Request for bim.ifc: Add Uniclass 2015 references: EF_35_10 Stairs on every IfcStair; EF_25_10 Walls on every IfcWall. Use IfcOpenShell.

First a look at what the model holds.

```python
import ifcopenshell

model = ifcopenshell.open("bim.ifc")
print(model.schema)
print("classifications:", [c.Name for c in model.by_type("IfcClassification")])
for ifc_class in ("IfcDoor", "IfcRoof", "IfcStair", "IfcWall", "IfcWindow"):
    print(ifc_class, len(model.by_type(ifc_class)))
```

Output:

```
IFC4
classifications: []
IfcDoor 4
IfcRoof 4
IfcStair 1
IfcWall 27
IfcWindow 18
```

```python
import ifcopenshell
import ifcopenshell.api.classification

model = ifcopenshell.open("bim.ifc")

system = ifcopenshell.api.classification.add_classification(model, classification="Uniclass 2015")

codes = {
    "IfcStair": ("EF_35_10", "Stairs"),
    "IfcWall": ("EF_25_10", "Walls"),
}
for ifc_class, (code, name) in codes.items():
    products = model.by_type(ifc_class)
    ifcopenshell.api.classification.add_reference(
        model, products=products, classification=system, identification=code, name=name
    )
    print(code, len(products))

model.write("bim_updated.ifc")
```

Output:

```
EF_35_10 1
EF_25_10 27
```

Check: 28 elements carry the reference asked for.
